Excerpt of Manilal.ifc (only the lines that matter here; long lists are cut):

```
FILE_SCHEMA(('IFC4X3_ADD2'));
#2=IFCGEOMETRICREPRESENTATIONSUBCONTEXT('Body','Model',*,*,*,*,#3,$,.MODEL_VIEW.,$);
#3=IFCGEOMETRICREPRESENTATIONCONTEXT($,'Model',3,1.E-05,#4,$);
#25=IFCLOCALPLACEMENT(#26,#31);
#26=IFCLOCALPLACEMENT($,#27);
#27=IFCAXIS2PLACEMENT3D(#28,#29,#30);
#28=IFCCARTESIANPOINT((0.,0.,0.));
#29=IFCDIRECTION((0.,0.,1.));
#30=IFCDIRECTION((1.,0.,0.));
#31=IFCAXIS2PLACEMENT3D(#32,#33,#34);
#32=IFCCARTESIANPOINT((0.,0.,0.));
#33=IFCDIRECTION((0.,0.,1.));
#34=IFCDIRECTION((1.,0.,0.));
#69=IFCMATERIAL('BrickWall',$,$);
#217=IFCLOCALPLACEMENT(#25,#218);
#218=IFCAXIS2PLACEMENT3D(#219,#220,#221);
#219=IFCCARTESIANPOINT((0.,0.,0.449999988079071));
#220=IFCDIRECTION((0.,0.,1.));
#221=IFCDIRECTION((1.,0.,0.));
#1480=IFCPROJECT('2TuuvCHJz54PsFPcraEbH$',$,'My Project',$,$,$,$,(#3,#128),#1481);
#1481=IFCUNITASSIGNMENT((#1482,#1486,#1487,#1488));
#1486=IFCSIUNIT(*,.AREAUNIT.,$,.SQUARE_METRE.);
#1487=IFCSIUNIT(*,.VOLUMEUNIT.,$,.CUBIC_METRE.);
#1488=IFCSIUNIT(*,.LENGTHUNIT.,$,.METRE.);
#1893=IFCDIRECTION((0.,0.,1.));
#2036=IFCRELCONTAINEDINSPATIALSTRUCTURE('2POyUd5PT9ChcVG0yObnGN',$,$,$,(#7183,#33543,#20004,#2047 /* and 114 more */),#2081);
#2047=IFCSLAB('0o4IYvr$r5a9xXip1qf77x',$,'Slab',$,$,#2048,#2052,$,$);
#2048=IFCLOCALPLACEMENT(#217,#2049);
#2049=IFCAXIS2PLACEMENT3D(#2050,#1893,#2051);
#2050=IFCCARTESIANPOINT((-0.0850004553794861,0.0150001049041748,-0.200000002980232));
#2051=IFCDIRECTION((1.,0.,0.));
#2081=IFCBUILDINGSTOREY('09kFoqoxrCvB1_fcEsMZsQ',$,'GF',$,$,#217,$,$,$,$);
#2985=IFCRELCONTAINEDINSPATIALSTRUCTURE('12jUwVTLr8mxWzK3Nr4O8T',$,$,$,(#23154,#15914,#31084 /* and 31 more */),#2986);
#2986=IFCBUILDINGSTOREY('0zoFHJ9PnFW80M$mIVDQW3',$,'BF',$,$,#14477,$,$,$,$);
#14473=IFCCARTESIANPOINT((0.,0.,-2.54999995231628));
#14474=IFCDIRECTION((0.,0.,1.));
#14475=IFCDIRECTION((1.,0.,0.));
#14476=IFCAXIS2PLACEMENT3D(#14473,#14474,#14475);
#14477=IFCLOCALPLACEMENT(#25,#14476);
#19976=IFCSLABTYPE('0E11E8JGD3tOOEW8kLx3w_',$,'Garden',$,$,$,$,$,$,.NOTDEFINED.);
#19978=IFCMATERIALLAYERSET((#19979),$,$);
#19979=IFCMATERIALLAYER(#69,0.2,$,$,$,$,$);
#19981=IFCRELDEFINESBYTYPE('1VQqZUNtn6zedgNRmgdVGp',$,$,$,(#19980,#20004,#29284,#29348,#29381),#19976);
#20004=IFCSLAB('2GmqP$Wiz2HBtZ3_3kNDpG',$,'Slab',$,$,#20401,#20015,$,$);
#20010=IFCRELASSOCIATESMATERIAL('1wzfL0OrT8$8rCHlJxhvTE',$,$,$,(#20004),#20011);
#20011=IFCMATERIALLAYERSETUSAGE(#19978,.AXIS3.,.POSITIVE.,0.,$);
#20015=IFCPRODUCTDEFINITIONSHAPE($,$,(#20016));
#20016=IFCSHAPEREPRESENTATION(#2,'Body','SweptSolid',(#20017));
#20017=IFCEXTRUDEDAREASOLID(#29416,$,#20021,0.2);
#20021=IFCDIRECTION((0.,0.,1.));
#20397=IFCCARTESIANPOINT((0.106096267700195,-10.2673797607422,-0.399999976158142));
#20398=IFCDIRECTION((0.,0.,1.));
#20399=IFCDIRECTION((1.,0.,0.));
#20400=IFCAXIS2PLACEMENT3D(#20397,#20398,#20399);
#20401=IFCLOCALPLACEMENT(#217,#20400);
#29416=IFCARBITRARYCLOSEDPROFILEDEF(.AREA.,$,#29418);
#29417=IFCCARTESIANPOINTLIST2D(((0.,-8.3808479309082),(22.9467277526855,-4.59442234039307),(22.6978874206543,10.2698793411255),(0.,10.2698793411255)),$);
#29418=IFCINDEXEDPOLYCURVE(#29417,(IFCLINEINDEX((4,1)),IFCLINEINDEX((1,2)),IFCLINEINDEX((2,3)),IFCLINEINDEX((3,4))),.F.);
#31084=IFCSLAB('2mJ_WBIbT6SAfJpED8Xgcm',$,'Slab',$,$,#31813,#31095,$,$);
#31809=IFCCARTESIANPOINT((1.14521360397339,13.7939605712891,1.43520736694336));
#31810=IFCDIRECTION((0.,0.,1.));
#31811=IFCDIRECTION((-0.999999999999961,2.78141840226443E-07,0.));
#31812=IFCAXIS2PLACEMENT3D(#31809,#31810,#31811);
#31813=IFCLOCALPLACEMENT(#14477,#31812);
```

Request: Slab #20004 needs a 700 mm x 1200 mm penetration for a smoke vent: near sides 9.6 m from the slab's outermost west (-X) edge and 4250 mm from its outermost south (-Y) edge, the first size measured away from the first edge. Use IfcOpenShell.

```python
import numpy as np
import ifcopenshell
import ifcopenshell.api.feature
import ifcopenshell.api.geometry
import ifcopenshell.api.root
import ifcopenshell.geom
import ifcopenshell.util.placement
import ifcopenshell.util.representation
import ifcopenshell.util.shape
import ifcopenshell.util.unit

model = ifcopenshell.open("Manilal.ifc")
unit_scale = ifcopenshell.util.unit.calculate_unit_scale(model)
settings = ifcopenshell.geom.settings()


def volume(element):
    """Net volume in cubic metres, openings subtracted."""
    shape = ifcopenshell.geom.create_shape(settings, element)
    return ifcopenshell.util.shape.get_volume(shape.geometry)


slab = model.by_guid("2GmqP$Wiz2HBtZ3_3kNDpG")
before = volume(slab)

# Extent in the slab's own axes, in metres. The edges named are its -X and -Y sides.
slab_shape = ifcopenshell.geom.create_shape(settings, slab)
vertices = ifcopenshell.util.shape.get_vertices(slab_shape.geometry)
x_min, y_min, bottom = vertices.min(axis=0)
top = vertices[:, 2].max()

opening = ifcopenshell.api.root.create_entity(model, ifc_class="IfcOpeningElement", name="Smoke vent opening", predefined_type="OPENING")
context = ifcopenshell.util.representation.get_context(model, "Model", "Body", "MODEL_VIEW")
width, depth = 0.7, 1.2
outline = [(0.0, 0.0), (width, 0.0), (width, depth), (0.0, depth), (0.0, 0.0)]
# Overshoot both faces by 50 mm so the cut is clean.
shape = ifcopenshell.api.geometry.add_slab_representation(
    model, context=context, depth=top - bottom + 0.1, polyline=outline
)
ifcopenshell.api.geometry.assign_representation(model, product=opening, representation=shape)

matrix = ifcopenshell.util.placement.get_local_placement(slab.ObjectPlacement)
matrix[:, 3] = matrix @ np.append(np.array([x_min + 9.6, y_min + 4.25, bottom - 0.05]) / unit_scale, 1.0)
ifcopenshell.api.geometry.edit_object_placement(model, product=opening, matrix=matrix, is_si=False)
ifcopenshell.api.feature.add_feature(model, feature=opening, element=slab)

after = volume(slab)

print(f"slab volume {before:.3f} -> {after:.3f} m3")

model.write("Manilal-out.ifc")
```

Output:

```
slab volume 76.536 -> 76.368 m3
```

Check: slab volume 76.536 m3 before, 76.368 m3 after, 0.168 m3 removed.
